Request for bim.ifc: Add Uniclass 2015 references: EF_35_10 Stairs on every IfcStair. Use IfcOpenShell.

First a look at what the model holds.

```python
import ifcopenshell

model = ifcopenshell.open("bim.ifc")
print(model.schema)
print("classifications:", [c.Name for c in model.by_type("IfcClassification")])
for ifc_class in ("IfcDoor", "IfcRoof", "IfcStair", "IfcWall", "IfcWindow"):
    print(ifc_class, len(model.by_type(ifc_class)))
```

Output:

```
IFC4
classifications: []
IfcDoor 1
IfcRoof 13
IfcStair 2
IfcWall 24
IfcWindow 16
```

```python
import ifcopenshell
import ifcopenshell.api.classification

model = ifcopenshell.open("bim.ifc")

system = ifcopenshell.api.classification.add_classification(model, classification="Uniclass 2015")

codes = {
    "IfcStair": ("EF_35_10", "Stairs"),
}
for ifc_class, (code, name) in codes.items():
    products = model.by_type(ifc_class)
    ifcopenshell.api.classification.add_reference(
        model, products=products, classification=system, identification=code, name=name
    )
    print(code, len(products))

model.write("bim_rev.ifc")
```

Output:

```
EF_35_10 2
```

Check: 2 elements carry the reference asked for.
